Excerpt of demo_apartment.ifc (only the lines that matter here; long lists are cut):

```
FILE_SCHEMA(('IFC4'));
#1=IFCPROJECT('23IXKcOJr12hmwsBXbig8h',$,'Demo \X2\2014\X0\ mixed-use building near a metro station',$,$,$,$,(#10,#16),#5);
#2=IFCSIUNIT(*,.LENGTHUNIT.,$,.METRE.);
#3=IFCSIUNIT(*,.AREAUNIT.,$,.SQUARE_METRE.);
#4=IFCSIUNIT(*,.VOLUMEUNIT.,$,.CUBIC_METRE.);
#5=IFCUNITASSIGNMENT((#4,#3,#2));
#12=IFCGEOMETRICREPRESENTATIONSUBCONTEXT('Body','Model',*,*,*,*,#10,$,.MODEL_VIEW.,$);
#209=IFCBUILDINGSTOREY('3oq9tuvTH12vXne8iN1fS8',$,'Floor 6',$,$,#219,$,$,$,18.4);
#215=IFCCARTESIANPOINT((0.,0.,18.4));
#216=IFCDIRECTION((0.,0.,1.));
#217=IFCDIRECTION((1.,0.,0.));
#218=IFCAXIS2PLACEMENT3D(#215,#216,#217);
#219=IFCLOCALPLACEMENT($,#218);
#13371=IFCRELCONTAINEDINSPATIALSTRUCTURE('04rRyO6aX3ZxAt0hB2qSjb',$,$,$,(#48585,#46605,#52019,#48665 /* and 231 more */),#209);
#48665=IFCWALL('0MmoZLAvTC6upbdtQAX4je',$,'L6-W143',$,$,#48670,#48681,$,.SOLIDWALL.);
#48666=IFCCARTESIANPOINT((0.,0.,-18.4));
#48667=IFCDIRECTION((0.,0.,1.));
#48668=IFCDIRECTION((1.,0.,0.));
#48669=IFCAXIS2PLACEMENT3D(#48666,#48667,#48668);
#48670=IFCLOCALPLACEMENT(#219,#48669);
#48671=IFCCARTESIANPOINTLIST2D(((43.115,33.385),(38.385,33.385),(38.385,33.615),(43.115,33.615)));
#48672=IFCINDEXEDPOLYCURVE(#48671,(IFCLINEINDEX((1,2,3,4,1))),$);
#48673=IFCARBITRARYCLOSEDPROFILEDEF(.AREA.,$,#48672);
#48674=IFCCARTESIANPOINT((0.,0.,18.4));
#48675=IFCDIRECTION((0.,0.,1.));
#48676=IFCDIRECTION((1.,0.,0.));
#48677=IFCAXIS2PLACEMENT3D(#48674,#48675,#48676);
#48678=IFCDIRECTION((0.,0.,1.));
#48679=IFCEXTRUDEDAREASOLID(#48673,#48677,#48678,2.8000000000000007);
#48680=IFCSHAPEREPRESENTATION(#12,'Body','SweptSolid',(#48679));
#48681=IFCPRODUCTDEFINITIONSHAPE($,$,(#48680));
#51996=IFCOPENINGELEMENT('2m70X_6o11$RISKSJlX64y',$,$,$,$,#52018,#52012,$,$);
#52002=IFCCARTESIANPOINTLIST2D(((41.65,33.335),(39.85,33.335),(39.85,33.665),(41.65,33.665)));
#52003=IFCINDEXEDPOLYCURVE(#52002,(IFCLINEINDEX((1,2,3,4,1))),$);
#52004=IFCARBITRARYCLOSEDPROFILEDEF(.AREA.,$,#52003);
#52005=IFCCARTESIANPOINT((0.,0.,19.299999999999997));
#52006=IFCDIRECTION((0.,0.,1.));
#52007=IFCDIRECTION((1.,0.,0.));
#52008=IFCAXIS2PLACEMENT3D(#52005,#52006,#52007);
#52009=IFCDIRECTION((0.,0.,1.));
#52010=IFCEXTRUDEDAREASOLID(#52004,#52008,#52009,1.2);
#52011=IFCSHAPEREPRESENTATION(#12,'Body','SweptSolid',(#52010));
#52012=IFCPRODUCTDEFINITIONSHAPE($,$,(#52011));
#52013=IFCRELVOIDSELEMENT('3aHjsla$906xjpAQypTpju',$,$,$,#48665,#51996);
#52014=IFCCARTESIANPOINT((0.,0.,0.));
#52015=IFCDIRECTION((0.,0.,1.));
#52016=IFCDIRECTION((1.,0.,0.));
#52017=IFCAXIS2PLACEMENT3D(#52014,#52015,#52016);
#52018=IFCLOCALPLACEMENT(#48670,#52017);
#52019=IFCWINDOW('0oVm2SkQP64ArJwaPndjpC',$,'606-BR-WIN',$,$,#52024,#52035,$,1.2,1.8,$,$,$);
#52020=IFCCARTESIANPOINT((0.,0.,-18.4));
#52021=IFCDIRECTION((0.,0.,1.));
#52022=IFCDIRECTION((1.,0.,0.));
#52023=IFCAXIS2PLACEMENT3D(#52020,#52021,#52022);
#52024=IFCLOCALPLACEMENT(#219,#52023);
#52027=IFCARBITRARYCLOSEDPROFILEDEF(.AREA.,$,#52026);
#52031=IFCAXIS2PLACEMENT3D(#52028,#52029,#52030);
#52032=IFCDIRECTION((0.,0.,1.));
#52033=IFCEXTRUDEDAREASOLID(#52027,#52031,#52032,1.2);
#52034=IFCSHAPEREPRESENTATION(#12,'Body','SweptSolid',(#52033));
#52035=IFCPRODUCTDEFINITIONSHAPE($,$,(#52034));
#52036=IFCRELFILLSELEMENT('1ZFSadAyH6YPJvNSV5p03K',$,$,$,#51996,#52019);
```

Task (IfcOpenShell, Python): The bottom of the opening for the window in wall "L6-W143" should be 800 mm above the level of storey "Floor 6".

```python
import numpy as np
import ifcopenshell
import ifcopenshell.api.geometry
import ifcopenshell.geom
import ifcopenshell.util.element
import ifcopenshell.util.placement
import ifcopenshell.util.shape
import ifcopenshell.util.unit

model = ifcopenshell.open("demo_apartment.ifc")
unit_scale = ifcopenshell.util.unit.calculate_unit_scale(model)

window = model.by_guid("0oVm2SkQP64ArJwaPndjpC")
opening = window.FillsVoids[0].RelatingOpeningElement
storey = ifcopenshell.util.element.get_container(window, ifc_class="IfcBuildingStorey")
level = ifcopenshell.util.placement.get_local_placement(storey.ObjectPlacement)[2, 3]

# The opening's origin need not be at the sill, so measure its lowest point.
shape = ifcopenshell.geom.create_shape(ifcopenshell.geom.settings(), opening)
bottom = ifcopenshell.util.shape.get_shape_bottom_elevation(shape, shape.geometry) / unit_scale
dz = level + 0.8 - bottom

shift = np.array([0.0, 0.0, dz])
# The window is not placed relative to its opening, so move both.
for product in (opening, window):
    matrix = ifcopenshell.util.placement.get_local_placement(product.ObjectPlacement)
    matrix[:3, 3] += shift
    ifcopenshell.api.geometry.edit_object_placement(model, product=product, matrix=matrix, is_si=False)

print(f"moved by {dz * unit_scale:+.3f} m")

model.write("demo_apartment_rev.ifc")
```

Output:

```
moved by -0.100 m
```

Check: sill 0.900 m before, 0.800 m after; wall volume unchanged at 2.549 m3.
